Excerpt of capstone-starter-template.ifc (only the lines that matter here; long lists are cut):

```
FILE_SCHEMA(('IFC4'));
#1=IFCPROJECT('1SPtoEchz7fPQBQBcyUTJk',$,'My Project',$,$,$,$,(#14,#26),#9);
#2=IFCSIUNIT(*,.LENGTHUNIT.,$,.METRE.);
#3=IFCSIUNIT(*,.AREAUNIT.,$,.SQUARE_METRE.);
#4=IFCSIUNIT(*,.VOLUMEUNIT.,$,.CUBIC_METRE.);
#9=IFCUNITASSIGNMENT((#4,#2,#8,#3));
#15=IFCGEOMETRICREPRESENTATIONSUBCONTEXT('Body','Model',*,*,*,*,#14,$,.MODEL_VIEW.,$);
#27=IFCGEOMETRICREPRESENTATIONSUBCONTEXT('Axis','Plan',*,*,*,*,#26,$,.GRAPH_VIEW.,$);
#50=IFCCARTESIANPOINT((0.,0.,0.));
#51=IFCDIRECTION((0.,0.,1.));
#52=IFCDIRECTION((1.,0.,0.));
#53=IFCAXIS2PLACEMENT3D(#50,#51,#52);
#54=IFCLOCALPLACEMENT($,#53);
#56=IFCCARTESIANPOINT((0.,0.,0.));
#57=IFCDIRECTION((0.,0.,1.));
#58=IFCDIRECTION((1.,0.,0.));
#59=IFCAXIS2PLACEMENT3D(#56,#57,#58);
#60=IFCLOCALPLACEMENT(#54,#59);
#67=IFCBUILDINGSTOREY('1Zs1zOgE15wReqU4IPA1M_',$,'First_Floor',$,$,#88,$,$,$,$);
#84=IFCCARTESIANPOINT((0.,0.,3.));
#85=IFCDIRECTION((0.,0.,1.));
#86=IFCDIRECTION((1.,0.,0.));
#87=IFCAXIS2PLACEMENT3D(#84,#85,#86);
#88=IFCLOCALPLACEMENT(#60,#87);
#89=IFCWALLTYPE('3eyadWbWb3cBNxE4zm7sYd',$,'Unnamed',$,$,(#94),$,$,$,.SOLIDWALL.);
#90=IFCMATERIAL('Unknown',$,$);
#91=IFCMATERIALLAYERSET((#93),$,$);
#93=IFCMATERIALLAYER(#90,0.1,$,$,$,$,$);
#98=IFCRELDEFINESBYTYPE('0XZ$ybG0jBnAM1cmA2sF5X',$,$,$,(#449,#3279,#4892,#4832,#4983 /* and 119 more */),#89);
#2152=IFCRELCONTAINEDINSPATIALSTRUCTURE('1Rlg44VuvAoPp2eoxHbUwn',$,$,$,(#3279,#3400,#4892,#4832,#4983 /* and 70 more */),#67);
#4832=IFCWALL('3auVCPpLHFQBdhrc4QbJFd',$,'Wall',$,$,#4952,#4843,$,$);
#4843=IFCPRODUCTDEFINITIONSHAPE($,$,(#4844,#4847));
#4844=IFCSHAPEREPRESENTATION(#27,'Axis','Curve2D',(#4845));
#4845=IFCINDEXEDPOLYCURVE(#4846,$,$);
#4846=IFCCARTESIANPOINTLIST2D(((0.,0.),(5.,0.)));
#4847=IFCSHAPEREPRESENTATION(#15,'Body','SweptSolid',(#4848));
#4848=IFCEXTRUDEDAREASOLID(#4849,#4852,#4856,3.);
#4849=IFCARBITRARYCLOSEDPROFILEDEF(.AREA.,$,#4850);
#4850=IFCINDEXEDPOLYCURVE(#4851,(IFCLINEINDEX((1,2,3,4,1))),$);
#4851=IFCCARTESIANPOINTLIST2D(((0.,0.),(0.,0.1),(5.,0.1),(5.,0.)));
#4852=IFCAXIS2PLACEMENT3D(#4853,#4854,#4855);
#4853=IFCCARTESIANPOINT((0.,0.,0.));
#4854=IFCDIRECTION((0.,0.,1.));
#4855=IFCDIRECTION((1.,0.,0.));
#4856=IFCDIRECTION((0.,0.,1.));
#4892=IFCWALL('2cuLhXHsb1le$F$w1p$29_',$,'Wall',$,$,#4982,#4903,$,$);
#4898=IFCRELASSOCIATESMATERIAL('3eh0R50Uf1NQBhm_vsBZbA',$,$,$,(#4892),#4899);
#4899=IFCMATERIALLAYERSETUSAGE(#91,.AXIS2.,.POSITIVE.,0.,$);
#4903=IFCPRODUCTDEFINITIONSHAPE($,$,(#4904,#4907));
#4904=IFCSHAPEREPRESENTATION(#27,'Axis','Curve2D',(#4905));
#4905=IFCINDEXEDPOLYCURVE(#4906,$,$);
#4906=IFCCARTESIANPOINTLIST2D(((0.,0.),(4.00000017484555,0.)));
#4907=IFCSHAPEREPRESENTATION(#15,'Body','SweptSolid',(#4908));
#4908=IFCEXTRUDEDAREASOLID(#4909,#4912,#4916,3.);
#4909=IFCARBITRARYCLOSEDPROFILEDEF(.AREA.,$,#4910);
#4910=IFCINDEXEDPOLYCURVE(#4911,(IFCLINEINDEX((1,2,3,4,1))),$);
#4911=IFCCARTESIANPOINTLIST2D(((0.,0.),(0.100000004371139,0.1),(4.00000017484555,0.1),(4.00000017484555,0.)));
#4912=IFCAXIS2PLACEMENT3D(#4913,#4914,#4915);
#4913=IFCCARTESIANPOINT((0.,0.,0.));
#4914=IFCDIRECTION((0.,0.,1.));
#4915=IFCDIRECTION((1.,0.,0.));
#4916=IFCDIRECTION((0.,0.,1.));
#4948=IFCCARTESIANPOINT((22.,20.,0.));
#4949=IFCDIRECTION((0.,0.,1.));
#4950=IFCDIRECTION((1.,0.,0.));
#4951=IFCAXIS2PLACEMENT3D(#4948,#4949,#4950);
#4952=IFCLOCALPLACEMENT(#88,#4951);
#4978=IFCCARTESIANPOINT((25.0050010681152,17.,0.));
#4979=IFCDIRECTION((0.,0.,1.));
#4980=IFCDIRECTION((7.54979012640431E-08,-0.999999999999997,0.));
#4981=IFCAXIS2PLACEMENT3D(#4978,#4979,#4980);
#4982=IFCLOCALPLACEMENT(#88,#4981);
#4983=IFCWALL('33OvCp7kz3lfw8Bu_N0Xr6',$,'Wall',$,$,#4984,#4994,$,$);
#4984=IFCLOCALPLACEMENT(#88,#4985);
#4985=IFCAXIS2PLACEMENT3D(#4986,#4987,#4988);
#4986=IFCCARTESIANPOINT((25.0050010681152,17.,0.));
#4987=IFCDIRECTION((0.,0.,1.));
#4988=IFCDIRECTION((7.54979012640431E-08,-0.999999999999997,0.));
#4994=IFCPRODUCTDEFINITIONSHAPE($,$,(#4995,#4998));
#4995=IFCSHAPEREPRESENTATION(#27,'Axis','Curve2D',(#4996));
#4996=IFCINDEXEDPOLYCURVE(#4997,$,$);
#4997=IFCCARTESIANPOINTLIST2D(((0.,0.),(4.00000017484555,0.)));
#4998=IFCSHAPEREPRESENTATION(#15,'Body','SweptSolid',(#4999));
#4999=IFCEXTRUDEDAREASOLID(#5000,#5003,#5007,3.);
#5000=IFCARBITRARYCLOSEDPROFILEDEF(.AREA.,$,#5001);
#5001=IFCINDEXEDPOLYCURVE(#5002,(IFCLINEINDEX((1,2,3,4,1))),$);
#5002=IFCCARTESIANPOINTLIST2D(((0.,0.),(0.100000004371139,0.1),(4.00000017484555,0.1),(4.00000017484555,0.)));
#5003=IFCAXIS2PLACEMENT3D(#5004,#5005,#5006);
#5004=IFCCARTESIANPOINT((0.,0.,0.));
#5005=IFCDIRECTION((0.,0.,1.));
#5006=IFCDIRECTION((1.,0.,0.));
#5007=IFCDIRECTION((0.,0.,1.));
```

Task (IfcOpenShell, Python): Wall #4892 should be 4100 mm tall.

```python
import ifcopenshell
import ifcopenshell.geom
import ifcopenshell.util.representation
import ifcopenshell.util.shape

model = ifcopenshell.open("capstone-starter-template.ifc")
settings = ifcopenshell.geom.settings()


def volume(element):
    """Net volume in cubic metres, openings subtracted."""
    shape = ifcopenshell.geom.create_shape(settings, element)
    return ifcopenshell.util.shape.get_volume(shape.geometry)


wall = model.by_guid("2cuLhXHsb1le$F$w1p$29_")
before = volume(wall)

body = ifcopenshell.util.representation.get_representation(wall, "Model", "Body")
solid = body.Items[0]
old_height = solid.Depth
solid.Depth = 4.1
after = volume(wall)

print(f"height {old_height:g} -> {solid.Depth:g}, volume {before:.3f} -> {after:.3f} m3")

model.write("capstone-starter-template-out.ifc")
```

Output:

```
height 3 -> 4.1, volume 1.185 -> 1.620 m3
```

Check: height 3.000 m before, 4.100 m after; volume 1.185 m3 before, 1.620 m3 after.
